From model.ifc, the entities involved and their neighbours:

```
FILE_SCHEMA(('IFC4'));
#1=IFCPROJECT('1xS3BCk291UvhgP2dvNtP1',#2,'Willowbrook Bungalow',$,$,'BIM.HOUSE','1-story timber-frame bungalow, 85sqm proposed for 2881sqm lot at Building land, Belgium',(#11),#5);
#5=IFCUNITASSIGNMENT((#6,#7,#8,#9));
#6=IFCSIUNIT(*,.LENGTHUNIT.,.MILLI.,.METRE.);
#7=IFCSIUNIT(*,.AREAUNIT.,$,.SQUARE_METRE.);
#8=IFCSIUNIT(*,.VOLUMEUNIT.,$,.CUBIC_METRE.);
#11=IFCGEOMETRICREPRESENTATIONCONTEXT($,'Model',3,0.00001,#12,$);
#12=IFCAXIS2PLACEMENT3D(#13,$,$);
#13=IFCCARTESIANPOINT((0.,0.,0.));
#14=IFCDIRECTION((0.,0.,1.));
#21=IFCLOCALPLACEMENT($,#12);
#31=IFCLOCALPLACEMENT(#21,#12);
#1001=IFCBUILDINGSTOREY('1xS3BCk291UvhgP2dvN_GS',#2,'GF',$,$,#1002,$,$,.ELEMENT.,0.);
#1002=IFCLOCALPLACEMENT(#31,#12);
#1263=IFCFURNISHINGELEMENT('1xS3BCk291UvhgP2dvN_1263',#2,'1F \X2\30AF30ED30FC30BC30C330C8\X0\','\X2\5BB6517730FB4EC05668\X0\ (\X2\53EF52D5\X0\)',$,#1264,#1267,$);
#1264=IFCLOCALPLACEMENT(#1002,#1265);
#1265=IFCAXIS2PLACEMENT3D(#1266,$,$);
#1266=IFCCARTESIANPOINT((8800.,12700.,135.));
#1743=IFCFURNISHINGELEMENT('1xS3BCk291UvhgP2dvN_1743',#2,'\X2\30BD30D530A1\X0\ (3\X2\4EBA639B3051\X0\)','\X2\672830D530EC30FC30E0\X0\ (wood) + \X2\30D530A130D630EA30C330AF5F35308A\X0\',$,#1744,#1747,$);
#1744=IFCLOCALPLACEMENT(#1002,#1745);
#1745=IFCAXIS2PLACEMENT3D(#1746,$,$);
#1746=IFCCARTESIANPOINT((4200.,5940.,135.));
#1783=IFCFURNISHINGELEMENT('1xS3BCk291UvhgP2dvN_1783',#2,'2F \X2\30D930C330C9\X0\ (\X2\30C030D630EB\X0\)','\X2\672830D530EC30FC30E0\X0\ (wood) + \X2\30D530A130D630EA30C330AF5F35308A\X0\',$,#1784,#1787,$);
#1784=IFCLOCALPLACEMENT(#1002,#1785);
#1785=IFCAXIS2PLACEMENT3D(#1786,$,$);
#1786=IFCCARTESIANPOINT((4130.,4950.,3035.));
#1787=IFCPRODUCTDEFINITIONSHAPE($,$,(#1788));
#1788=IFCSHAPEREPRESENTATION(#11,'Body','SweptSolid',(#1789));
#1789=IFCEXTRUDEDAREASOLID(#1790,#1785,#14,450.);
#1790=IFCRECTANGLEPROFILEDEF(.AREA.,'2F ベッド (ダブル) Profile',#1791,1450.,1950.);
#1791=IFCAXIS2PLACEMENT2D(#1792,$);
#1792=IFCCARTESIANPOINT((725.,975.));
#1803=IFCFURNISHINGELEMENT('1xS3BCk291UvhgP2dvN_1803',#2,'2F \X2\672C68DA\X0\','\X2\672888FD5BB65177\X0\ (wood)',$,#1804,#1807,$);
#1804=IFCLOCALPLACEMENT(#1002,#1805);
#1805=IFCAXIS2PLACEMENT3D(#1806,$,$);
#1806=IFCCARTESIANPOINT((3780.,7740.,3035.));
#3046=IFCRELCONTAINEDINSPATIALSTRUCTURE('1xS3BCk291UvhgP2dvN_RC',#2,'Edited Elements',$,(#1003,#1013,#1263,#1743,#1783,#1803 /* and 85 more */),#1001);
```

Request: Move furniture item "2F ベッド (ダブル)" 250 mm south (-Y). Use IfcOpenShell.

```python
import ifcopenshell
import ifcopenshell.api.geometry
import ifcopenshell.util.placement
import ifcopenshell.util.unit

model = ifcopenshell.open("model.ifc")
unit_scale = ifcopenshell.util.unit.calculate_unit_scale(model)

item = model.by_guid("1xS3BCk291UvhgP2dvN_1783")
matrix = ifcopenshell.util.placement.get_local_placement(item.ObjectPlacement)
matrix[1, 3] -= 0.25 / unit_scale
ifcopenshell.api.geometry.edit_object_placement(model, product=item, matrix=matrix, is_si=False)

print(ifcopenshell.util.placement.get_local_placement(item.ObjectPlacement).round(3) + 0.0)

model.write("model_rev.ifc")
```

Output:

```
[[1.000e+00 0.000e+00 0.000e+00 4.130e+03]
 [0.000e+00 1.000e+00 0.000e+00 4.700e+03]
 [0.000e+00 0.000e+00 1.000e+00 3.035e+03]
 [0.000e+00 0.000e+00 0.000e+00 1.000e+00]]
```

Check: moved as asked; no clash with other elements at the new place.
